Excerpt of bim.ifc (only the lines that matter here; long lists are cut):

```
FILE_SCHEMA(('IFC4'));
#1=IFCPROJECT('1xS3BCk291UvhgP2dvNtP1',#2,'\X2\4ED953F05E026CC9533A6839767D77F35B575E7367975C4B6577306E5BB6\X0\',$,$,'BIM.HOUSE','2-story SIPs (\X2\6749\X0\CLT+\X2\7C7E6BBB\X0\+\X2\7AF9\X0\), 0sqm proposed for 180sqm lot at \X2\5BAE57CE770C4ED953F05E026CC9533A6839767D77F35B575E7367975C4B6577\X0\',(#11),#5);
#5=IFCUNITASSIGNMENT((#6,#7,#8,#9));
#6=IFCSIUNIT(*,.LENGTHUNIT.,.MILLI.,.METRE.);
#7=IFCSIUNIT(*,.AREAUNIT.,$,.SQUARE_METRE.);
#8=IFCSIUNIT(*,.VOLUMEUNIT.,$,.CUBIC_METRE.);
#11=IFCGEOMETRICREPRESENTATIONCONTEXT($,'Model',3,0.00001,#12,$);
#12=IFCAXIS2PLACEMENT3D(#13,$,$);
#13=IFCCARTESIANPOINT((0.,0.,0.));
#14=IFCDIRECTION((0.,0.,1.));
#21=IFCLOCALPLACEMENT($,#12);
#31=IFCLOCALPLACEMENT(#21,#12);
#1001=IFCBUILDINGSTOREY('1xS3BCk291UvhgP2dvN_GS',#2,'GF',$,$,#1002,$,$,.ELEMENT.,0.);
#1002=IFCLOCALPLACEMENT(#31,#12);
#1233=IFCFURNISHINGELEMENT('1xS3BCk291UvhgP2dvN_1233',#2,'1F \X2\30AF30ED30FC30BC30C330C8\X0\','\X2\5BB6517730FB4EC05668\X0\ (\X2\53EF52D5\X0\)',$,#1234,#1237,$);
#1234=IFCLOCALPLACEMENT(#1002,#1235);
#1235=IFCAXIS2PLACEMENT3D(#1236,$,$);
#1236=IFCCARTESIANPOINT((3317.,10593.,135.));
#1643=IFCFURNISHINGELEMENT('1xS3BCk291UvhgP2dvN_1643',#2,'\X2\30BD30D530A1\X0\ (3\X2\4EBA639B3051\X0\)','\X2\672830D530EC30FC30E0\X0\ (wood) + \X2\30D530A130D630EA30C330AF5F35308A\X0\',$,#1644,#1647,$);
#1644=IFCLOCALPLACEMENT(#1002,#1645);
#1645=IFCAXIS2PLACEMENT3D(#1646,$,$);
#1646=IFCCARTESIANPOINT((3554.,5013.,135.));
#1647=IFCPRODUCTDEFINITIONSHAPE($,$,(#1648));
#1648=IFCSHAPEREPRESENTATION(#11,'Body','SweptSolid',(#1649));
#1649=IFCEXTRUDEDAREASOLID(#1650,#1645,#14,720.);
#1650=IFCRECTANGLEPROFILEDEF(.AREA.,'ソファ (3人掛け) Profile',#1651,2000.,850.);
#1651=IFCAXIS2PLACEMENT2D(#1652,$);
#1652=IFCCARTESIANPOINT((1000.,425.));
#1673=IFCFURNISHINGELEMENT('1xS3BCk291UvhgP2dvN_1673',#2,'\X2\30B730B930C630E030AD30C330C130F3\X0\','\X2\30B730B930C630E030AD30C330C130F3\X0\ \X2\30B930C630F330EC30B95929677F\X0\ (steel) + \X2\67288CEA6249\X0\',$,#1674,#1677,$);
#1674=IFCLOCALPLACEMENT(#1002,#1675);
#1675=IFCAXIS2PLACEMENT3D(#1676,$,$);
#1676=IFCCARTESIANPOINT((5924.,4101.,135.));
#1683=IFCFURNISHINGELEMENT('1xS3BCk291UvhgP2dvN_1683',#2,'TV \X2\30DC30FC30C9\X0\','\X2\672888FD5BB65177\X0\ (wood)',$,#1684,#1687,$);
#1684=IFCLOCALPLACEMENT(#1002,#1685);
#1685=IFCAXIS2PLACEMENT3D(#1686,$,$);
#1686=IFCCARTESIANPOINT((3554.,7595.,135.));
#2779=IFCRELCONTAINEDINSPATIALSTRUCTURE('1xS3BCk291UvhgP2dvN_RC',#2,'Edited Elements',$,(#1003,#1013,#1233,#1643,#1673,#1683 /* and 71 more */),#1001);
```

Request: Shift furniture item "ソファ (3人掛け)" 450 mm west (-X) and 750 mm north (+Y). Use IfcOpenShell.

```python
import ifcopenshell
import ifcopenshell.api.geometry
import ifcopenshell.util.placement
import ifcopenshell.util.unit

model = ifcopenshell.open("bim.ifc")
unit_scale = ifcopenshell.util.unit.calculate_unit_scale(model)

item = model.by_guid("1xS3BCk291UvhgP2dvN_1643")
matrix = ifcopenshell.util.placement.get_local_placement(item.ObjectPlacement)
matrix[0, 3] -= 0.45 / unit_scale
matrix[1, 3] += 0.75 / unit_scale
ifcopenshell.api.geometry.edit_object_placement(model, product=item, matrix=matrix, is_si=False)

print(ifcopenshell.util.placement.get_local_placement(item.ObjectPlacement).round(3) + 0.0)

model.write("bim_v2.ifc")
```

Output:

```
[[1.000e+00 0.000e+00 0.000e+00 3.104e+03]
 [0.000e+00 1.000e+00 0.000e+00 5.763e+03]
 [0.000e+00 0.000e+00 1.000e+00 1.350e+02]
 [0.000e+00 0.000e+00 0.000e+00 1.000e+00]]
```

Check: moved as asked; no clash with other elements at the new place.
